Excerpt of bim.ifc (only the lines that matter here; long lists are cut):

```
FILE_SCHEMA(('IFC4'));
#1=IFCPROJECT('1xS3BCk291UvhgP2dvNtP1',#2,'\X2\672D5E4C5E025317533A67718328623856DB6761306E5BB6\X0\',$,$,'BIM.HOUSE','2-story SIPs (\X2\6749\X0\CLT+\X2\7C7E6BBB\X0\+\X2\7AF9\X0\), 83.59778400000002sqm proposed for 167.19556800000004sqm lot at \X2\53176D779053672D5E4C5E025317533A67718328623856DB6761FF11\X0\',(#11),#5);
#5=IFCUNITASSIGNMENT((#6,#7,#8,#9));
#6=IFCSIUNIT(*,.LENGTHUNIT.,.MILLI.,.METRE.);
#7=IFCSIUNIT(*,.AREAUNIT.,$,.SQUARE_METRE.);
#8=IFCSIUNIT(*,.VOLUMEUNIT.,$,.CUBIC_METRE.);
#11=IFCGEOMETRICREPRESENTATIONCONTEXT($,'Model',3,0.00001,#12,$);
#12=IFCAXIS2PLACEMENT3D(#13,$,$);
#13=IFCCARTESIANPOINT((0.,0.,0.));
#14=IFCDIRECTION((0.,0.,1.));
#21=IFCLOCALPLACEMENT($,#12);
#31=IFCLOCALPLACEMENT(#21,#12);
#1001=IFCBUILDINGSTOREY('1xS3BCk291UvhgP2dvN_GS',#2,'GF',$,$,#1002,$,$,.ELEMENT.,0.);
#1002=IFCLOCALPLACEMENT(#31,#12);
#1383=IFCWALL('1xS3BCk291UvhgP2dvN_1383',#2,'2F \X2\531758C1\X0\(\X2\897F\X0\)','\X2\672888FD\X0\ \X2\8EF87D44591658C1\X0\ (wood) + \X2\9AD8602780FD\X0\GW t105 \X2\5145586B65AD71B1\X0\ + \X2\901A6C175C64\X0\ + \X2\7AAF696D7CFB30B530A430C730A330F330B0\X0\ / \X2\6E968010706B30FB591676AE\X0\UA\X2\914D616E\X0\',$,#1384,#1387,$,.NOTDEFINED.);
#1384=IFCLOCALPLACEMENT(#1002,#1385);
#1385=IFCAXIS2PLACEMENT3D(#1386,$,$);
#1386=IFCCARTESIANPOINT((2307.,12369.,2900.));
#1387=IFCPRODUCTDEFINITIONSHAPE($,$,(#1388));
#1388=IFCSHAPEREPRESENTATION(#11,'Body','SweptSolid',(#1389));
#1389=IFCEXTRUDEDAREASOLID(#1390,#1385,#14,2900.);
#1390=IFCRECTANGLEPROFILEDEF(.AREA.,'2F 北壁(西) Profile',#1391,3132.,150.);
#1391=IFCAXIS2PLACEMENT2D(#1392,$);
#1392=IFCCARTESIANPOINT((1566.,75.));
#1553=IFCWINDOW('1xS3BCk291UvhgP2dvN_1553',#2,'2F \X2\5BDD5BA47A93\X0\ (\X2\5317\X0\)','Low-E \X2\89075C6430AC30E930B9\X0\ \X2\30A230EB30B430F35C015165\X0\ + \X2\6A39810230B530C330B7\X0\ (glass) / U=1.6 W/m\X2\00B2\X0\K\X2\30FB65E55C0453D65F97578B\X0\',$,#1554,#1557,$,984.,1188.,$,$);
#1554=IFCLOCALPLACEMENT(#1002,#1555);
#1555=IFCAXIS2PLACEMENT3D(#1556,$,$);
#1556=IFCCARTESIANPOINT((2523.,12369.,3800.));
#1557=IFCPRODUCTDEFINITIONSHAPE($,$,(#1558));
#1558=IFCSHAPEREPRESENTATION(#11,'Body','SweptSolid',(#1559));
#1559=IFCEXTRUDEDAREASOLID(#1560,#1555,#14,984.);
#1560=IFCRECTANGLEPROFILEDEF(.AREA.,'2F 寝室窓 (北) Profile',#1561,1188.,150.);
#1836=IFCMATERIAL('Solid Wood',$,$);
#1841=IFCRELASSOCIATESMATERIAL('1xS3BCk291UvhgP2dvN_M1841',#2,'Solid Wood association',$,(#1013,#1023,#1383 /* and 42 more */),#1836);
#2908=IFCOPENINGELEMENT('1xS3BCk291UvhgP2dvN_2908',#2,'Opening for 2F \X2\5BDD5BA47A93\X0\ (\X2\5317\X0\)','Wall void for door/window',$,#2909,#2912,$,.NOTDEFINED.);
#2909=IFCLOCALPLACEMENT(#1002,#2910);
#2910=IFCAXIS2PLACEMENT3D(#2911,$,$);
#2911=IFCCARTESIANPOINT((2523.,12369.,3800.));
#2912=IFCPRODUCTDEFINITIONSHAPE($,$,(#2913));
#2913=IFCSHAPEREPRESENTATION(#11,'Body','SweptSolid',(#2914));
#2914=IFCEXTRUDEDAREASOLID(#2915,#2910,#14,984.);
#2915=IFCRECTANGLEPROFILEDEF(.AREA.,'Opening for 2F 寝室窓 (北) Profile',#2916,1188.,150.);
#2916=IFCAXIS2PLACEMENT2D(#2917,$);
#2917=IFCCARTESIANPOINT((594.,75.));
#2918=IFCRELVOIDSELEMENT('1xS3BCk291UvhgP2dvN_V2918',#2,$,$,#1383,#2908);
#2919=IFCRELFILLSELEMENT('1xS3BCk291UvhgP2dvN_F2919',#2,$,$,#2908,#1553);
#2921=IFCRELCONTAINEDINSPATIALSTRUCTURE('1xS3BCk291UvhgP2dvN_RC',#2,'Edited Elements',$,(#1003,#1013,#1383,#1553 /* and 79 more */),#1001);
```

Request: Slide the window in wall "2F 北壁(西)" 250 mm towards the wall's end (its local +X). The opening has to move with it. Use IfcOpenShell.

```python
import ifcopenshell
import ifcopenshell.api.geometry
import ifcopenshell.util.placement
import ifcopenshell.util.unit

model = ifcopenshell.open("bim.ifc")
unit_scale = ifcopenshell.util.unit.calculate_unit_scale(model)

window = model.by_guid("1xS3BCk291UvhgP2dvN_1553")
opening = window.FillsVoids[0].RelatingOpeningElement
wall = opening.VoidsElements[0].RelatingBuildingElement

wall_matrix = ifcopenshell.util.placement.get_local_placement(wall.ObjectPlacement)
shift = wall_matrix[:3, 0] * 0.25 / unit_scale
before = ifcopenshell.util.placement.get_local_placement(window.ObjectPlacement)[:3, 3].copy()

# The window is not placed relative to its opening, so move both.
for product in (opening, window):
    matrix = ifcopenshell.util.placement.get_local_placement(product.ObjectPlacement)
    matrix[:3, 3] += shift
    ifcopenshell.api.geometry.edit_object_placement(model, product=product, matrix=matrix, is_si=False)

after = ifcopenshell.util.placement.get_local_placement(window.ObjectPlacement)[:3, 3]
print("window moved by", (after - before).round(3) + 0.0)

model.write("bim_edited.ifc")
```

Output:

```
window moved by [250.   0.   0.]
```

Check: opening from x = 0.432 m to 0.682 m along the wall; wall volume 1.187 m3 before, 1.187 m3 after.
